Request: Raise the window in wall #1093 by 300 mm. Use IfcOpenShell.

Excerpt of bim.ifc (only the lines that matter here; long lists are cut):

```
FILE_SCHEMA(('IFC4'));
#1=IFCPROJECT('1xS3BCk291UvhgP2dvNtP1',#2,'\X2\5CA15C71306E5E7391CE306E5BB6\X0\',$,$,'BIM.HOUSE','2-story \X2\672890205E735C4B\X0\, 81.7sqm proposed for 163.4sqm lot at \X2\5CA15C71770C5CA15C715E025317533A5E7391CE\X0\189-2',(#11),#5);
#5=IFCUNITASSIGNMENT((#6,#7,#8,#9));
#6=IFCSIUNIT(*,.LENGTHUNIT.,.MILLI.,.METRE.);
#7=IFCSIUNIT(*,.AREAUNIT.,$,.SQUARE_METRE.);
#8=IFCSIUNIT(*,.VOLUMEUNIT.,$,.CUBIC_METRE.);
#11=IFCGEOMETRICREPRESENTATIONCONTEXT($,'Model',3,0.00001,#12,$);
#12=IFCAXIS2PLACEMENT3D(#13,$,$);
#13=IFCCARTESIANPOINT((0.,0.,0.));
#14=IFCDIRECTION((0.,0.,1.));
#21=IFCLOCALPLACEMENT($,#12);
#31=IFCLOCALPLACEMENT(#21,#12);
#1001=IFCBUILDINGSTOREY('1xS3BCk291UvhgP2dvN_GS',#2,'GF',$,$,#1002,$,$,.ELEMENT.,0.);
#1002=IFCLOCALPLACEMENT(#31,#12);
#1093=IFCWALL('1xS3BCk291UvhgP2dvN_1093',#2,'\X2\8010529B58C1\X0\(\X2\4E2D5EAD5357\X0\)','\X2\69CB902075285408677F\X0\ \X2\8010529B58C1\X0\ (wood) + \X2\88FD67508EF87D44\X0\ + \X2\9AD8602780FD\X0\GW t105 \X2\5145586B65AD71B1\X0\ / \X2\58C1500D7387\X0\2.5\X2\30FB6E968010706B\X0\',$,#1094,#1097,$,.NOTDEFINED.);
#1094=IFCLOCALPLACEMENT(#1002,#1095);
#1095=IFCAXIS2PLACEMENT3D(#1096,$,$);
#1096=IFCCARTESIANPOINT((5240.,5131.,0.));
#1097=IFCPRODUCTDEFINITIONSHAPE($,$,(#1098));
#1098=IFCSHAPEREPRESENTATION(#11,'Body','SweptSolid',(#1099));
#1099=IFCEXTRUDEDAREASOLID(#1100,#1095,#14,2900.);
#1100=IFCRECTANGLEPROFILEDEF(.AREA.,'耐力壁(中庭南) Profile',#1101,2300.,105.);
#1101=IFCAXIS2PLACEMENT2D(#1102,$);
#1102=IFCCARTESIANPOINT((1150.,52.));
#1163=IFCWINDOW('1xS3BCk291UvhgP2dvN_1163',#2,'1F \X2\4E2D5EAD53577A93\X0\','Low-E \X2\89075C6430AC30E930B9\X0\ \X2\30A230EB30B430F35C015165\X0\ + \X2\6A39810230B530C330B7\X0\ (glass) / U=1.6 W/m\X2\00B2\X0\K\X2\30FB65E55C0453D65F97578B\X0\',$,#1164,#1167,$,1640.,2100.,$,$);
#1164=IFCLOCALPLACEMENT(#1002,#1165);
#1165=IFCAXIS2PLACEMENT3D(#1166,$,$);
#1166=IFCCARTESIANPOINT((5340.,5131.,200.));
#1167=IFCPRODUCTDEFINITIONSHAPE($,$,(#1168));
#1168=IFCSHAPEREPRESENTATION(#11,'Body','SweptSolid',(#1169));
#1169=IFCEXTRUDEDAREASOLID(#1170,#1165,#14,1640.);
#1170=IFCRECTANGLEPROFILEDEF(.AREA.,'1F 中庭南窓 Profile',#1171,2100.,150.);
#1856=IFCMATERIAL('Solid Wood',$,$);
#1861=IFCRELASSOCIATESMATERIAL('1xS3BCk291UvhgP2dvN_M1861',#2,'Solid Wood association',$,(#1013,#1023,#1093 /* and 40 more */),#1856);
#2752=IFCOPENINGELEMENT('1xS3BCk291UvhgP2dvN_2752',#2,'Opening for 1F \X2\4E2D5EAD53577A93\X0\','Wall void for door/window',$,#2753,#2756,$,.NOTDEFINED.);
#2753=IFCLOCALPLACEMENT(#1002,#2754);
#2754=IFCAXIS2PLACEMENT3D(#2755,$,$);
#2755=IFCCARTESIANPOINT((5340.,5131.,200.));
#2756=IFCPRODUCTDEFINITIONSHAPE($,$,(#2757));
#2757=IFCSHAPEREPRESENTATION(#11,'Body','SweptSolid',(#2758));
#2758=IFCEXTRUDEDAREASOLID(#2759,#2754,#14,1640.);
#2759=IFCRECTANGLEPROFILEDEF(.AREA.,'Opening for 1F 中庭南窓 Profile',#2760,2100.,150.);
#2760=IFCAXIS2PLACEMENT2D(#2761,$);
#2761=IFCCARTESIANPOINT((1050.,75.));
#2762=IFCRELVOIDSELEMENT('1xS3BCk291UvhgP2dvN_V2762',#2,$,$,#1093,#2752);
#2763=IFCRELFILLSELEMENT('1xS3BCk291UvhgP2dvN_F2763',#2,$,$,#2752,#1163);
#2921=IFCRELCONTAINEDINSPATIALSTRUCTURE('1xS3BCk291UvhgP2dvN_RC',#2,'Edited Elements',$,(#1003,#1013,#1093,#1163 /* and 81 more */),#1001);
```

```python
import numpy as np
import ifcopenshell
import ifcopenshell.api.geometry
import ifcopenshell.util.placement
import ifcopenshell.util.unit

model = ifcopenshell.open("bim.ifc")
unit_scale = ifcopenshell.util.unit.calculate_unit_scale(model)

window = model.by_guid("1xS3BCk291UvhgP2dvN_1163")
opening = window.FillsVoids[0].RelatingOpeningElement
dz = 300.0

shift = np.array([0.0, 0.0, dz])
# The window is not placed relative to its opening, so move both.
for product in (opening, window):
    matrix = ifcopenshell.util.placement.get_local_placement(product.ObjectPlacement)
    matrix[:3, 3] += shift
    ifcopenshell.api.geometry.edit_object_placement(model, product=product, matrix=matrix, is_si=False)

print(f"moved by {dz * unit_scale:+.3f} m")

model.write("bim_edited.ifc")
```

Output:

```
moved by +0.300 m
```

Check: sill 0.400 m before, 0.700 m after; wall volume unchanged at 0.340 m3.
